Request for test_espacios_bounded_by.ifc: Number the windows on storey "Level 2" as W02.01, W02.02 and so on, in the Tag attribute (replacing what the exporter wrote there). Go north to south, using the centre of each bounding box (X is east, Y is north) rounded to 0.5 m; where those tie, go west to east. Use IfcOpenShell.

First a look at what the model holds.

```python
import ifcopenshell
import ifcopenshell.util.element
import ifcopenshell.util.placement

model = ifcopenshell.open("test_espacios_bounded_by.ifc")
print(model.schema)
storey = next(s for s in model.by_type("IfcBuildingStorey") if s.Name == "Level 2")
windows = [e for e in ifcopenshell.util.element.get_decomposition(storey) if e.is_a("IfcWindow")]
for e in sorted(windows, key=lambda e: e.id()):
    origin = ifcopenshell.util.placement.get_local_placement(e.ObjectPlacement)[:3, 3]
    print(e.id(), e.Tag, e.Name, origin.round(2) + 0.0, sep=" | ")
```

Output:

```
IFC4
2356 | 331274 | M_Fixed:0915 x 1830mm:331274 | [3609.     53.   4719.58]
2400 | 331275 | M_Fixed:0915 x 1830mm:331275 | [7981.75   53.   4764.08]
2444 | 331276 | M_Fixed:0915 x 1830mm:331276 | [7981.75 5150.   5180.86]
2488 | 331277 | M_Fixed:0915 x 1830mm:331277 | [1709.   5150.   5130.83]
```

```python
import ifcopenshell
import ifcopenshell.geom
import ifcopenshell.util.element
import ifcopenshell.util.shape

model = ifcopenshell.open("test_espacios_bounded_by.ifc")
settings = ifcopenshell.geom.settings()
settings.set("use-world-coords", True)


def centre(element):
    shape = ifcopenshell.geom.create_shape(settings, element)
    return ifcopenshell.util.shape.get_bbox_centroid(shape.geometry)


storey = next(s for s in model.by_type("IfcBuildingStorey") if s.Name == "Level 2")
windows = [e for e in ifcopenshell.util.element.get_decomposition(storey) if e.is_a("IfcWindow")]

# Insertion points can sit at a corner or the storey origin, so sort by the geometry (in metres).
centres = {e: centre(e) for e in windows}
windows.sort(key=lambda e: (-round(centres[e][1] / 0.5), centres[e][0]))

for i, e in enumerate(windows, start=1):
    number = f"W02.{i:02d}"
    e.Tag = number
    print(e.id(), number)

model.write("test_espacios_bounded_by-out.ifc")
```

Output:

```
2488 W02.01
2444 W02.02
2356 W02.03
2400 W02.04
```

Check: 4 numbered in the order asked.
